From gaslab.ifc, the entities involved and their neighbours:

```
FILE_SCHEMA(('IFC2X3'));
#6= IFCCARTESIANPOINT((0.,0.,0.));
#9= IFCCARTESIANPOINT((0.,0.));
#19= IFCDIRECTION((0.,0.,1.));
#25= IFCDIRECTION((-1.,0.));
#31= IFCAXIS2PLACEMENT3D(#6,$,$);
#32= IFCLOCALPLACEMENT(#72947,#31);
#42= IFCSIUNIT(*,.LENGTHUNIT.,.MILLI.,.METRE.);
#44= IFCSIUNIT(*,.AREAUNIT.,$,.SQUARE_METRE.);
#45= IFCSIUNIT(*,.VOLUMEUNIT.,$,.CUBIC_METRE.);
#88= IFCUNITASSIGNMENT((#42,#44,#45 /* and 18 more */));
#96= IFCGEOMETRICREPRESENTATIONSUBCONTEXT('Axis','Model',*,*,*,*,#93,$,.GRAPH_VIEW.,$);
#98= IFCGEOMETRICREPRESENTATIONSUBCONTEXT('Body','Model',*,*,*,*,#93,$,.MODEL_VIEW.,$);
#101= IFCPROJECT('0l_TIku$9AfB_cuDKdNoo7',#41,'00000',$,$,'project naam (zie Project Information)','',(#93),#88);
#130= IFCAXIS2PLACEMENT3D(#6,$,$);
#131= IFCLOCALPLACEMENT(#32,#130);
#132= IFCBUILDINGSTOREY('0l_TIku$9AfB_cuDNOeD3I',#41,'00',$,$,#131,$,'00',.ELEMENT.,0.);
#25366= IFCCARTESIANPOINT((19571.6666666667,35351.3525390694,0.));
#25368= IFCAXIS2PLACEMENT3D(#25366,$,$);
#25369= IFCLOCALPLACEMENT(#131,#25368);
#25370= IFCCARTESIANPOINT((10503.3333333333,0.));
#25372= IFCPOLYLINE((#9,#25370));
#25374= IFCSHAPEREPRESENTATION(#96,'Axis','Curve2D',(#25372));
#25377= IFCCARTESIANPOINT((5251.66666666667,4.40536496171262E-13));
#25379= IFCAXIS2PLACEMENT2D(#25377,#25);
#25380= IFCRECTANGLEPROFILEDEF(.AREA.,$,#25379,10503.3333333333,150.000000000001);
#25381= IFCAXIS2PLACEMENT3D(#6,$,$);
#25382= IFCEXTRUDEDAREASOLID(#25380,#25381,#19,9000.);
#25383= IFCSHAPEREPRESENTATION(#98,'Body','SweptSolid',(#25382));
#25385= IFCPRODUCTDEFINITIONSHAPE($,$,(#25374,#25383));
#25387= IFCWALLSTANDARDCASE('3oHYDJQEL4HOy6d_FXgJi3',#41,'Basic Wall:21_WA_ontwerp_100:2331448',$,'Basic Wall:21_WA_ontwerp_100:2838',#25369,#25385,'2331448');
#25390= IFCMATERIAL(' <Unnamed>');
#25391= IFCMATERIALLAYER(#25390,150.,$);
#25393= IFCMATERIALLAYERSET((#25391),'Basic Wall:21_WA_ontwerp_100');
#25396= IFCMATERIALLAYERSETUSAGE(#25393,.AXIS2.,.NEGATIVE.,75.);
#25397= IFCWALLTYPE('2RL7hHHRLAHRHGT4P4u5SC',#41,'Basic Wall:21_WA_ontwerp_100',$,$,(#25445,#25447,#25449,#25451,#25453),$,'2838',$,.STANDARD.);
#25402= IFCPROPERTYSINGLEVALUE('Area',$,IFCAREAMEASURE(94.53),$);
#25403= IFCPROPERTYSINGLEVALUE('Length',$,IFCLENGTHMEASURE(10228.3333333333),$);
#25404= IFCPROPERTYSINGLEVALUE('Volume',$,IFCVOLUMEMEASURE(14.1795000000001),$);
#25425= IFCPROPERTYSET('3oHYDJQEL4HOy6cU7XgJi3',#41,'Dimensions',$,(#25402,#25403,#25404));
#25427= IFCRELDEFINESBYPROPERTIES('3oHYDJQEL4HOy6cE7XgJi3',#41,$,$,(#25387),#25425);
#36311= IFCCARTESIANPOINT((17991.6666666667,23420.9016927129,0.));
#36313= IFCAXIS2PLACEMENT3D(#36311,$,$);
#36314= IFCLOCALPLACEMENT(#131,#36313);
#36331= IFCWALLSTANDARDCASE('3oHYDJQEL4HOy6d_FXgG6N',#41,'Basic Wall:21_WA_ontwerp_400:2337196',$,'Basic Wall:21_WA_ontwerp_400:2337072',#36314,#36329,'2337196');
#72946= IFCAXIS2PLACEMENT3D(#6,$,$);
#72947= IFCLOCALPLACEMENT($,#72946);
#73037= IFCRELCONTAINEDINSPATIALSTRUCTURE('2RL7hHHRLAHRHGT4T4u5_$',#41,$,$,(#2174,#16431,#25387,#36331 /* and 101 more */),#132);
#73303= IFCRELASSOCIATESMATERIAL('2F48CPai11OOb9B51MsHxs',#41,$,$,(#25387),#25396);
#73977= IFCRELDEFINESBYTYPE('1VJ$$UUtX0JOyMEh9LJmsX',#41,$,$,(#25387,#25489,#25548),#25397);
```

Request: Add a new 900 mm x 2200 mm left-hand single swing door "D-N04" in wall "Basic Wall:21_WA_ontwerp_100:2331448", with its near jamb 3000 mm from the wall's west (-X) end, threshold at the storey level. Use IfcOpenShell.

```python
import numpy as np
import ifcopenshell
import ifcopenshell.api.feature
import ifcopenshell.api.geometry
import ifcopenshell.api.pset
import ifcopenshell.api.root
import ifcopenshell.api.spatial
import ifcopenshell.api.type
import ifcopenshell.geom
import ifcopenshell.util.element
import ifcopenshell.util.placement
import ifcopenshell.util.representation
import ifcopenshell.util.shape
import ifcopenshell.util.unit

model = ifcopenshell.open("gaslab.ifc")
unit_scale = ifcopenshell.util.unit.calculate_unit_scale(model)
area_scale = ifcopenshell.util.unit.calculate_unit_scale(model, "AREAUNIT")
volume_scale = ifcopenshell.util.unit.calculate_unit_scale(model, "VOLUMEUNIT")
settings = ifcopenshell.geom.settings()


def volume(element):
    """Net volume in cubic metres, openings subtracted."""
    shape = ifcopenshell.geom.create_shape(settings, element)
    return ifcopenshell.util.shape.get_volume(shape.geometry)


wall = model.by_guid("3oHYDJQEL4HOy6d_FXgJi3")
storey = ifcopenshell.util.element.get_container(wall, ifc_class="IfcBuildingStorey")
context = ifcopenshell.util.representation.get_context(model, "Model", "Body", "MODEL_VIEW")
before = volume(wall)

width, height, from_end, sill = 0.9, 2.2, 3, 0.0  # metres

# The wall runs along its own X axis, and the end named is its -X end.
wall_shape = ifcopenshell.geom.create_shape(settings, wall)
x, y, z = ifcopenshell.util.shape.get_vertices(wall_shape.geometry).T
start = x.min() + from_end
face, thickness = float(y.min()), float(y.max() - y.min())
wall_matrix = ifcopenshell.util.placement.get_local_placement(wall.ObjectPlacement)
level = ifcopenshell.util.placement.get_local_placement(storey.ObjectPlacement)[2, 3]


def in_wall(x, y):
    """Placement at x, y metres in the wall's axes, at sill height."""
    matrix = wall_matrix.copy()
    matrix[:, 3] = wall_matrix @ np.array([x / unit_scale, y / unit_scale, 0.0, 1.0])
    matrix[2, 3] = level + sill / unit_scale
    return matrix


# Opening: a box that overshoots both wall faces by 50 mm.
opening = ifcopenshell.api.root.create_entity(model, ifc_class="IfcOpeningElement")
box = ifcopenshell.api.geometry.add_wall_representation(
    model, context=context, length=width, height=height, thickness=thickness + 0.1
)
ifcopenshell.api.geometry.assign_representation(model, product=opening, representation=box)
ifcopenshell.api.geometry.edit_object_placement(model, product=opening, matrix=in_wall(start, face - 0.05), is_si=False)
ifcopenshell.api.feature.add_feature(model, feature=opening, element=wall)

door = ifcopenshell.api.root.create_entity(model, ifc_class="IfcDoor", name="D-N04")
door.OverallWidth, door.OverallHeight = width / unit_scale, height / unit_scale
body = ifcopenshell.api.geometry.add_door_representation(
    model,
    context=context,
    overall_width=door.OverallWidth,
    overall_height=door.OverallHeight,
    operation_type="SINGLE_SWING_LEFT",
    lining_properties={"LiningDepth": thickness / unit_scale, "ThresholdDepth": thickness / unit_scale},
)
ifcopenshell.api.geometry.assign_representation(model, product=door, representation=body)
ifcopenshell.api.spatial.assign_container(model, products=[door], relating_structure=storey)
fills = ifcopenshell.api.feature.add_filling(model, opening=opening, element=door)
fills.OwnerHistory = door.OwnerHistory  # required in IFC2X3

# IFC2X3 keeps the operation on the door style.
style = ifcopenshell.api.root.create_entity(model, ifc_class="IfcDoorStyle", name="D-N04")
style.OperationType, style.ConstructionType = "SINGLE_SWING_LEFT", "NOTDEFINED"
style.ParameterTakesPrecedence = style.Sizeable = False
ifcopenshell.api.type.assign_type(model, related_objects=[door], relating_type=style)

# The lining spans the wall, so the door starts at the wall face.
ifcopenshell.api.geometry.edit_object_placement(model, product=door, matrix=in_wall(start, face), is_si=False)

after = volume(wall)

# Update the wall's stored quantities.
pset = model.by_id(ifcopenshell.util.element.get_pset(wall, "Dimensions", should_inherit=False)["id"])
ifcopenshell.api.pset.edit_pset(model, pset=pset, properties={
    "Area": model.create_entity("IfcAreaMeasure", after / thickness / area_scale),
    "Volume": model.create_entity("IfcVolumeMeasure", after / volume_scale),
})

print(f"wall volume {before:.3f} -> {after:.3f} m3")

model.write("gaslab_updated.ifc")
```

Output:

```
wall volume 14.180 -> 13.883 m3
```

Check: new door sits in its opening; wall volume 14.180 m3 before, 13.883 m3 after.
